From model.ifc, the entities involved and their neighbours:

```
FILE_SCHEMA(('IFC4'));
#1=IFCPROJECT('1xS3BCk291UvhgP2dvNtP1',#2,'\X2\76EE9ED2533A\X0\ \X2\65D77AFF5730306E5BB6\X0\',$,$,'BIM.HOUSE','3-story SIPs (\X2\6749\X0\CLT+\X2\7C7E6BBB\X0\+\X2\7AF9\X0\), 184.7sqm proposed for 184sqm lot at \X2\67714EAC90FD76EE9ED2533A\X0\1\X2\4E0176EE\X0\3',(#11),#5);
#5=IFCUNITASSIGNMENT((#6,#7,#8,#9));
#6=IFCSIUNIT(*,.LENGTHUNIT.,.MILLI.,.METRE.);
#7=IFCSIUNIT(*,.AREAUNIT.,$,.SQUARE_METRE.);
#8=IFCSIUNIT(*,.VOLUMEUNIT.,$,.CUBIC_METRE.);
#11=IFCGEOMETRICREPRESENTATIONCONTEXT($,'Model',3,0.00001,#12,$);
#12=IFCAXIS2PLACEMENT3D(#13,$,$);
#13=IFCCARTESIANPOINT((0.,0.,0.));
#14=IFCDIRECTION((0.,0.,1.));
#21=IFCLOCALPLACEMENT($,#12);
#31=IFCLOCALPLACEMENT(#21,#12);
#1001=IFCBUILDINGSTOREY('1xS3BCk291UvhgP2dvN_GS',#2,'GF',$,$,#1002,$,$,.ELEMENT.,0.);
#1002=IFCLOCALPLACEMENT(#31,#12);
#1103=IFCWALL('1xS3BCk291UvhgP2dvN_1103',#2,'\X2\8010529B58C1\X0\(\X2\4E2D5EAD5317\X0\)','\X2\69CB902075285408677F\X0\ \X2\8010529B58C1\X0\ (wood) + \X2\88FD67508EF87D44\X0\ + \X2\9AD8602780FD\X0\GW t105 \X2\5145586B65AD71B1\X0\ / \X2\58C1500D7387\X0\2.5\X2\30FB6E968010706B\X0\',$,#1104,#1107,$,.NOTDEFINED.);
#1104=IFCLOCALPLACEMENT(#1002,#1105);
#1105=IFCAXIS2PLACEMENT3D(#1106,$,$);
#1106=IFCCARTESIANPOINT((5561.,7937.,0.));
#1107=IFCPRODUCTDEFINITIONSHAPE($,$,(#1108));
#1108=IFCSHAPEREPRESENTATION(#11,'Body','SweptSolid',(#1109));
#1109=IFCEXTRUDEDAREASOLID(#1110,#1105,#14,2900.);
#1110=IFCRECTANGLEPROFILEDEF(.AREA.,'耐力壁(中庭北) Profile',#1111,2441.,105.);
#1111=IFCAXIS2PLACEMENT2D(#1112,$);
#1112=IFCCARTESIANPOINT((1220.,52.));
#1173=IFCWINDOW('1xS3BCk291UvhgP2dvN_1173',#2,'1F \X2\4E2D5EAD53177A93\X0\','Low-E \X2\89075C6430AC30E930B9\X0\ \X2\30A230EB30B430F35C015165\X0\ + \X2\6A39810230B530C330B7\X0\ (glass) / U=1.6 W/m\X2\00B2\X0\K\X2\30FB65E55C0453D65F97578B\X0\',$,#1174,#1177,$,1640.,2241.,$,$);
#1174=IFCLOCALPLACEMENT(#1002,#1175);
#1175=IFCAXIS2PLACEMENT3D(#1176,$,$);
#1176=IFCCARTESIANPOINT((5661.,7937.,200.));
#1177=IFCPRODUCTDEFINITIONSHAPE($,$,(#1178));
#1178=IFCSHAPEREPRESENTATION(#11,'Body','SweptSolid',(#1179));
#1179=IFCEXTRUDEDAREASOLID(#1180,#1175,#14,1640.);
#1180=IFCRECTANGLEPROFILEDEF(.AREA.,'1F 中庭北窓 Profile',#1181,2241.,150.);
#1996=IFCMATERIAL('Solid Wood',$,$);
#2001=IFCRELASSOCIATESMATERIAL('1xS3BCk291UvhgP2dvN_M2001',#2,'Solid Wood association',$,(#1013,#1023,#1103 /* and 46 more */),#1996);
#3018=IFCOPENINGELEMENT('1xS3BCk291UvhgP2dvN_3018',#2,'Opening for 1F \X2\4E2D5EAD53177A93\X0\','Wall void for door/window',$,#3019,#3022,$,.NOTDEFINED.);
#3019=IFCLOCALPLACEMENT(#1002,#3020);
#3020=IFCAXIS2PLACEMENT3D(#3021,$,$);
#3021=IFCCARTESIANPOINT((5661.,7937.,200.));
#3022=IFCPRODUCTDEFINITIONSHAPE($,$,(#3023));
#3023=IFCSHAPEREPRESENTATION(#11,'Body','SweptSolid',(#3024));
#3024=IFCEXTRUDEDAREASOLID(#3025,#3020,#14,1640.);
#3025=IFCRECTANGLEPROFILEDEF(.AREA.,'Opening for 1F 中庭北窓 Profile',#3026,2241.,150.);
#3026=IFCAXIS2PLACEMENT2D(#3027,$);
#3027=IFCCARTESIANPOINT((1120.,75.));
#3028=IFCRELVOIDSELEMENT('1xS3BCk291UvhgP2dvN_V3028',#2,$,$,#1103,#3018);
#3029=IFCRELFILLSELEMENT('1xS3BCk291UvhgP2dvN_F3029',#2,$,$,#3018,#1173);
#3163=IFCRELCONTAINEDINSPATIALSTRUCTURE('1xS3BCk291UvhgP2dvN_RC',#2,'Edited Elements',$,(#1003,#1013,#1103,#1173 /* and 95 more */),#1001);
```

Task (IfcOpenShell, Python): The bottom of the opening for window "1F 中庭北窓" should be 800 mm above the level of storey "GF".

```python
import numpy as np
import ifcopenshell
import ifcopenshell.api.geometry
import ifcopenshell.geom
import ifcopenshell.util.element
import ifcopenshell.util.placement
import ifcopenshell.util.shape
import ifcopenshell.util.unit

model = ifcopenshell.open("model.ifc")
unit_scale = ifcopenshell.util.unit.calculate_unit_scale(model)

window = model.by_guid("1xS3BCk291UvhgP2dvN_1173")
opening = window.FillsVoids[0].RelatingOpeningElement
storey = ifcopenshell.util.element.get_container(window, ifc_class="IfcBuildingStorey")
level = ifcopenshell.util.placement.get_local_placement(storey.ObjectPlacement)[2, 3]

# The opening's origin need not be at the sill, so measure its lowest point.
shape = ifcopenshell.geom.create_shape(ifcopenshell.geom.settings(), opening)
bottom = ifcopenshell.util.shape.get_shape_bottom_elevation(shape, shape.geometry) / unit_scale
dz = level + 0.8 / unit_scale - bottom

shift = np.array([0.0, 0.0, dz])
# The window is not placed relative to its opening, so move both.
for product in (opening, window):
    matrix = ifcopenshell.util.placement.get_local_placement(product.ObjectPlacement)
    matrix[:3, 3] += shift
    ifcopenshell.api.geometry.edit_object_placement(model, product=product, matrix=matrix, is_si=False)

print(f"moved by {dz * unit_scale:+.3f} m")

model.write("model_updated.ifc")
```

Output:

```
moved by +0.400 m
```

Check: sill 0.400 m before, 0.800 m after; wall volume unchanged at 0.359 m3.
